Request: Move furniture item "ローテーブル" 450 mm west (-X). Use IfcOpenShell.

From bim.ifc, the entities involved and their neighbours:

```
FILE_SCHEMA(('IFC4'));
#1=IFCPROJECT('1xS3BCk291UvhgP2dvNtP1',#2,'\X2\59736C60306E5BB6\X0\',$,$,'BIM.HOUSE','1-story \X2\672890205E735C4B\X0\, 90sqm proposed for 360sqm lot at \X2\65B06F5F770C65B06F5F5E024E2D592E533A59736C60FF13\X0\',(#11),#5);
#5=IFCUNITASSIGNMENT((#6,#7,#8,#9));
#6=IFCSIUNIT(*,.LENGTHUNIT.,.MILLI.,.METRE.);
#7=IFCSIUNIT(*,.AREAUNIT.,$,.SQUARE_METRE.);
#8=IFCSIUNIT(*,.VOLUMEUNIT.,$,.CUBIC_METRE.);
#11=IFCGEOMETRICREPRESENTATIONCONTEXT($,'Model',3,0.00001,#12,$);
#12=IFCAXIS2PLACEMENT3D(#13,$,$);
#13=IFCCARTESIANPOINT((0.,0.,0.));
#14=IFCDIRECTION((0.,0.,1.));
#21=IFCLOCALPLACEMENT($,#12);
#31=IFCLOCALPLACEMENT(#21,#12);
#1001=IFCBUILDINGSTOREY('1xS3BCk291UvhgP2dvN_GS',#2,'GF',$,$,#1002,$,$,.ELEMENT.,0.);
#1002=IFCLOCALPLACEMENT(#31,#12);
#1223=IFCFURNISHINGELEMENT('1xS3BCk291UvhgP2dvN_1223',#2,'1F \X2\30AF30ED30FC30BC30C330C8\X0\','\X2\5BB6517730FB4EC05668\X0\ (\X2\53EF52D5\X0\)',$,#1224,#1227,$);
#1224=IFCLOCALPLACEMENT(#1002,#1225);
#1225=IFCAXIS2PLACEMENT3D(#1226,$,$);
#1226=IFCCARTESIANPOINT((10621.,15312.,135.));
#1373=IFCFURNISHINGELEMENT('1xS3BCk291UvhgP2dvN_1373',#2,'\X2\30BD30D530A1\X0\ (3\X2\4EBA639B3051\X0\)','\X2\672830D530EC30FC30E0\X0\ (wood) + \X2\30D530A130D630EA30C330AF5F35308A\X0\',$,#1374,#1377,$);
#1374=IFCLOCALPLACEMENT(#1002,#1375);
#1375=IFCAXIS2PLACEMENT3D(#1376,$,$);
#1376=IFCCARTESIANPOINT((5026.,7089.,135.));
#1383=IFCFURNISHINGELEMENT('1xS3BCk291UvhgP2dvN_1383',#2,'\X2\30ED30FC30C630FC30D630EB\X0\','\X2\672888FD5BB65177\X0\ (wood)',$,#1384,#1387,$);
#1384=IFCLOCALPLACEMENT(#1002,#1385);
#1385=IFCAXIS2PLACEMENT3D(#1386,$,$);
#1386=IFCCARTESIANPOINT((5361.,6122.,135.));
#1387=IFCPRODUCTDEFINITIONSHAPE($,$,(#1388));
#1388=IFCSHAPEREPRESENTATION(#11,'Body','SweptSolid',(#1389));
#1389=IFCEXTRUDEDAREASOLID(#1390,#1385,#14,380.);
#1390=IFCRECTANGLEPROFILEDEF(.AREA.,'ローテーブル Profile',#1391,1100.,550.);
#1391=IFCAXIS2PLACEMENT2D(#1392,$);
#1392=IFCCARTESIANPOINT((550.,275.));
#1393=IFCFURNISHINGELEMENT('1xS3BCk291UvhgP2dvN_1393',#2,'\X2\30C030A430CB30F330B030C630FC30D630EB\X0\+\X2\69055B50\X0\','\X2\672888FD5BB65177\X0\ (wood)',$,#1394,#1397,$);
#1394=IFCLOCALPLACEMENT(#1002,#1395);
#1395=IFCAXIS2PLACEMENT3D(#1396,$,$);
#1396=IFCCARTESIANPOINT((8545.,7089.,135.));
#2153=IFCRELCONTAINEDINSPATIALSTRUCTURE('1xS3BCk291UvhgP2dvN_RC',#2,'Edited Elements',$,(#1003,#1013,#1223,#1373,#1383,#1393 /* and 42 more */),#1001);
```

```python
import ifcopenshell
import ifcopenshell.api.geometry
import ifcopenshell.util.placement

model = ifcopenshell.open("bim.ifc")

item = model.by_guid("1xS3BCk291UvhgP2dvN_1383")
matrix = ifcopenshell.util.placement.get_local_placement(item.ObjectPlacement)
matrix[0, 3] -= 450.0
ifcopenshell.api.geometry.edit_object_placement(model, product=item, matrix=matrix, is_si=False)

print(ifcopenshell.util.placement.get_local_placement(item.ObjectPlacement).round(3) + 0.0)

model.write("bim_edited.ifc")
```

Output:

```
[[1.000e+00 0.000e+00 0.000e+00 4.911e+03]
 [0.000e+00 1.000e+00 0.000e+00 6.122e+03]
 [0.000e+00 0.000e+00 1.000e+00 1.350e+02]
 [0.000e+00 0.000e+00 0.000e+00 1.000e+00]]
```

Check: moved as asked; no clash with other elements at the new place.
